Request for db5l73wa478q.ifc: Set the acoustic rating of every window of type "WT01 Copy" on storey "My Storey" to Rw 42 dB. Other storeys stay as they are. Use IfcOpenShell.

First a look at what the model holds.

```python
import ifcopenshell
import ifcopenshell.util.element

model = ifcopenshell.open("db5l73wa478q.ifc")
print(model.schema)
storey = next(s for s in model.by_type("IfcBuildingStorey") if s.Name == "My Storey")
windows = [e for e in ifcopenshell.util.element.get_decomposition(storey) if e.is_a("IfcWindow")]
seen = {}
for e in windows:
    element_type = ifcopenshell.util.element.get_type(e)
    key = (element_type.Name if element_type != e and element_type else None, ifcopenshell.util.element.get_pset(e, "Pset_WindowCommon", "AcousticRating"))
    seen[key] = seen.get(key, 0) + 1
for (name, value), count in sorted(seen.items(), key=str):
    print(count, "x", name, "|", value)
```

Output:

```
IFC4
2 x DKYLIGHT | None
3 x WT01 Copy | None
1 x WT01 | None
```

```python
import ifcopenshell
import ifcopenshell.api.pset
import ifcopenshell.util.element

model = ifcopenshell.open("db5l73wa478q.ifc")

storey = next(s for s in model.by_type("IfcBuildingStorey") if s.Name == "My Storey")
windows = [e for e in ifcopenshell.util.element.get_decomposition(storey) if e.is_a("IfcWindow")]

count = 0
for e in windows:
    element_type = ifcopenshell.util.element.get_type(e)
    if element_type in (None, e) or element_type.Name != "WT01 Copy":
        continue
    # add_pset returns the element's existing set when there is one.
    pset = ifcopenshell.api.pset.add_pset(model, product=e, name="Pset_WindowCommon")
    ifcopenshell.api.pset.edit_pset(model, pset=pset, properties={"AcousticRating": "Rw 42 dB"})
    count += 1

print(count, "windows updated")

model.write("db5l73wa478q_rev.ifc")
```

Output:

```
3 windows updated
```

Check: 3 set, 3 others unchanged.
